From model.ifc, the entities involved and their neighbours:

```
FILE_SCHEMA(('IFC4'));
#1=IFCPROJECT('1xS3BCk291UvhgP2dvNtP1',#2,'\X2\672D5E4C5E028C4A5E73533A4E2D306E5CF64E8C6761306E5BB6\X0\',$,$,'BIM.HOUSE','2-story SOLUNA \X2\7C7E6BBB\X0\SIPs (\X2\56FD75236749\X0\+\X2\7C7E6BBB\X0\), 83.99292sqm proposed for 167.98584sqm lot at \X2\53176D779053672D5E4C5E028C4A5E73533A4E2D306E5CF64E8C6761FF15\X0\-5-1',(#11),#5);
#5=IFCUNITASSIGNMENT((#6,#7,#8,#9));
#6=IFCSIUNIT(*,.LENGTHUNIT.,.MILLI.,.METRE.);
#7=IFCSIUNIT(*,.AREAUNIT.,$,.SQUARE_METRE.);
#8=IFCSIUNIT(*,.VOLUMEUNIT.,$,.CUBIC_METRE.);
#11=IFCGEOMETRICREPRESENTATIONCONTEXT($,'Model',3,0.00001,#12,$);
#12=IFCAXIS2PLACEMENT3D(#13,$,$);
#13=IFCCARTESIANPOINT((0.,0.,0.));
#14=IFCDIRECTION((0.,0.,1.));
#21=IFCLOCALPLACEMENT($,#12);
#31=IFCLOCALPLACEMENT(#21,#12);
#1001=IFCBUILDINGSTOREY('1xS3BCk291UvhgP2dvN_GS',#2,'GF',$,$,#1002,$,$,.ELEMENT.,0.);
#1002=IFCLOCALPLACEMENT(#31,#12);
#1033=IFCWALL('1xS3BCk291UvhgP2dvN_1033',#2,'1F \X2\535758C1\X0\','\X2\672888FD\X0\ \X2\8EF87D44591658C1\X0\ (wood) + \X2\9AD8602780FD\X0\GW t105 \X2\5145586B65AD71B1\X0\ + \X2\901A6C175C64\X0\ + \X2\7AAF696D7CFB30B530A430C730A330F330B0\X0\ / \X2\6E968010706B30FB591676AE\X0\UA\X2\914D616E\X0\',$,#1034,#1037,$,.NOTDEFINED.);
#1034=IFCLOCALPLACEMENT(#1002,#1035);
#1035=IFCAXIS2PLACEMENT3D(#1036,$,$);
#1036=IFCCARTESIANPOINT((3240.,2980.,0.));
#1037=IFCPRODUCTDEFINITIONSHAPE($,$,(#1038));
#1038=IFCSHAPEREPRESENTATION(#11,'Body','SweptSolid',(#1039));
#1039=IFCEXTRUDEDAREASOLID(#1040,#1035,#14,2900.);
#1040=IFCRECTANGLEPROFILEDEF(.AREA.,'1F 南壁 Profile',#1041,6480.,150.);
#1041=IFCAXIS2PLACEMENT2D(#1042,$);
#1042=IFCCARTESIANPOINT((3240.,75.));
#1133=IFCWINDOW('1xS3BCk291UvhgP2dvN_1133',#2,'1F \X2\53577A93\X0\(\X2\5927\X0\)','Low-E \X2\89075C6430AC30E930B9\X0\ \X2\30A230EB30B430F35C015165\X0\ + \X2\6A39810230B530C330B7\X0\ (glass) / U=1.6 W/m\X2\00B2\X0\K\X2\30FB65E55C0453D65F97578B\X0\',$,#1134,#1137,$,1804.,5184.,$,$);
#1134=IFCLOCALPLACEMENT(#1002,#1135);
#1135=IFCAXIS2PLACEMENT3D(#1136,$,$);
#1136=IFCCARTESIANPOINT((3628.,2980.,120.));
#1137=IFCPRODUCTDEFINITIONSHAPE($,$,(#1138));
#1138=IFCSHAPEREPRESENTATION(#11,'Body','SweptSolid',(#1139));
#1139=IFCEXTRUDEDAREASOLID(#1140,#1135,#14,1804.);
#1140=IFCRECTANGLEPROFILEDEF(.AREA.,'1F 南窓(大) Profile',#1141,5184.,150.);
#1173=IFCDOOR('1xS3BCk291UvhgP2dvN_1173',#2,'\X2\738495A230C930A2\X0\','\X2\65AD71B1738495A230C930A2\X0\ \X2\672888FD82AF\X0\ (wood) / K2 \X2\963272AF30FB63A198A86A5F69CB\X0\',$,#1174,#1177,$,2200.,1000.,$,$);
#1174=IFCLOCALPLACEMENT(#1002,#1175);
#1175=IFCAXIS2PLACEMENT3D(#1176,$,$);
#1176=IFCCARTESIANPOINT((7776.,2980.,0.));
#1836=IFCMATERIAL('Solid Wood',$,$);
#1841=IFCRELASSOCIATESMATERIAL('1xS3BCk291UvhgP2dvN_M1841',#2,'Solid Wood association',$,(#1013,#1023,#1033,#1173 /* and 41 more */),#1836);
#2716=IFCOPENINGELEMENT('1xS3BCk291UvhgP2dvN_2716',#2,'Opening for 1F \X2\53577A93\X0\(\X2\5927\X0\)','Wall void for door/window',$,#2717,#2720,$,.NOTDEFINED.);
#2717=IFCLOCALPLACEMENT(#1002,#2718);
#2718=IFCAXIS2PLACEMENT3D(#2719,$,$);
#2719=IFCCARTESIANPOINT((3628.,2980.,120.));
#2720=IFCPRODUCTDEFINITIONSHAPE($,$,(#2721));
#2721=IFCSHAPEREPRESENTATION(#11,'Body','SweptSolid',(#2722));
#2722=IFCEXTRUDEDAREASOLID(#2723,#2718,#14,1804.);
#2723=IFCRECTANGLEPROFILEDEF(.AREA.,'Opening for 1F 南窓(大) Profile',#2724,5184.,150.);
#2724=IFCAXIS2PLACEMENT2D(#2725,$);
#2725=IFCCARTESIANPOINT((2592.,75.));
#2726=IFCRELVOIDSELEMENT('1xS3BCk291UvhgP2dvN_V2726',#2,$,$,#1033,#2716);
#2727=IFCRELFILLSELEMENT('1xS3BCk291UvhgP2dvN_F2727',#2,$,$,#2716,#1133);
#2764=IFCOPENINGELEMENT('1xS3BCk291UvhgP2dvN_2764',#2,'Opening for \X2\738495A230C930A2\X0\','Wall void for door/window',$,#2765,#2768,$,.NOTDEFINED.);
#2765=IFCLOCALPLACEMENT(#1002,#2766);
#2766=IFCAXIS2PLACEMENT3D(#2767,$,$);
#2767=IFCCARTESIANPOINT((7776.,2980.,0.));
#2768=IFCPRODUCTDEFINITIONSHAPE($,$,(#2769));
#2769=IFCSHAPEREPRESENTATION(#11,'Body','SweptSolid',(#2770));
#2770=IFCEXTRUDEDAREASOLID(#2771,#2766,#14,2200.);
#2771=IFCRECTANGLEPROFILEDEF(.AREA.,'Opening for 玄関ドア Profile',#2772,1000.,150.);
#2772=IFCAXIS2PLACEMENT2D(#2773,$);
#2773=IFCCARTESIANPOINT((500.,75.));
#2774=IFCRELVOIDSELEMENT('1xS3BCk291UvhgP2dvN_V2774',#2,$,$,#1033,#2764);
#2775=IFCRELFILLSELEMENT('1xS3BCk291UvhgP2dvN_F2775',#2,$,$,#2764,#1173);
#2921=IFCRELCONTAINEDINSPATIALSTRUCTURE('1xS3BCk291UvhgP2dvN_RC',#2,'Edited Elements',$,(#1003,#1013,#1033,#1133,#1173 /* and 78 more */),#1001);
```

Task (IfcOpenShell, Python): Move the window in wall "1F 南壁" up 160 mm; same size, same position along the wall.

```python
import numpy as np
import ifcopenshell
import ifcopenshell.api.geometry
import ifcopenshell.util.placement
import ifcopenshell.util.unit

model = ifcopenshell.open("model.ifc")
unit_scale = ifcopenshell.util.unit.calculate_unit_scale(model)

window = model.by_guid("1xS3BCk291UvhgP2dvN_1133")
opening = window.FillsVoids[0].RelatingOpeningElement
dz = 0.16 / unit_scale

shift = np.array([0.0, 0.0, dz])
# The window is not placed relative to its opening, so move both.
for product in (opening, window):
    matrix = ifcopenshell.util.placement.get_local_placement(product.ObjectPlacement)
    matrix[:3, 3] += shift
    ifcopenshell.api.geometry.edit_object_placement(model, product=product, matrix=matrix, is_si=False)

print(f"moved by {dz * unit_scale:+.3f} m")

model.write("model_v2.ifc")
```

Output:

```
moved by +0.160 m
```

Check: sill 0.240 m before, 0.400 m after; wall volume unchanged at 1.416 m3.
